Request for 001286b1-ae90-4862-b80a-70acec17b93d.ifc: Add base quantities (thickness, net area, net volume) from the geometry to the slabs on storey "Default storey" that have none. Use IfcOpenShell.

First a look at what the model holds.

```python
import ifcopenshell
import ifcopenshell.util.element
import ifcopenshell.util.unit

model = ifcopenshell.open("001286b1-ae90-4862-b80a-70acec17b93d.ifc")
print(model.schema)
for unit_type in ("LENGTHUNIT", "AREAUNIT", "VOLUMEUNIT"):
    print(unit_type, ifcopenshell.util.unit.calculate_unit_scale(model, unit_type))
storey = next(s for s in model.by_type("IfcBuildingStorey") if s.Name == "Default storey")
slabs = [e for e in ifcopenshell.util.element.get_decomposition(storey) if e.is_a("IfcSlab")]
for e in sorted(slabs, key=lambda e: e.id()):
    print(e.id(), e.is_a(), e.Name, list(ifcopenshell.util.element.get_psets(e, qtos_only=True)), sep=" | ")
```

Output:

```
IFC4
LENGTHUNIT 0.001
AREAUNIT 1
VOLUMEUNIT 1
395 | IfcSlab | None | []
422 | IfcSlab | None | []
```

```python
import ifcopenshell
import ifcopenshell.api.pset
import ifcopenshell.geom
import ifcopenshell.util.element
import ifcopenshell.util.shape
import ifcopenshell.util.unit

model = ifcopenshell.open("001286b1-ae90-4862-b80a-70acec17b93d.ifc")
unit_scale = ifcopenshell.util.unit.calculate_unit_scale(model)
area_scale = ifcopenshell.util.unit.calculate_unit_scale(model, "AREAUNIT")
volume_scale = ifcopenshell.util.unit.calculate_unit_scale(model, "VOLUMEUNIT")
settings = ifcopenshell.geom.settings()

storey = next(s for s in model.by_type("IfcBuildingStorey") if s.Name == "Default storey")
slabs = [e for e in ifcopenshell.util.element.get_decomposition(storey) if e.is_a("IfcSlab")]

for e in sorted(slabs, key=lambda e: e.id()):
    if ifcopenshell.util.element.get_psets(e, qtos_only=True, should_inherit=False):
        continue
    # Geometry comes back in metres, in the element's own axes.
    shape = ifcopenshell.geom.create_shape(settings, e)
    values = {
        "Width": ifcopenshell.util.shape.get_z(shape.geometry) / unit_scale,
        "NetArea": ifcopenshell.util.shape.get_footprint_area(shape.geometry) / area_scale,
        "NetVolume": ifcopenshell.util.shape.get_volume(shape.geometry) / volume_scale,
    }
    qto = ifcopenshell.api.pset.add_qto(model, product=e, name="Qto_SlabBaseQuantities")
    ifcopenshell.api.pset.edit_qto(model, qto=qto, properties=values)
    print(e.id(), {k: round(v, 3) for k, v in values.items()})

model.write("001286b1-ae90-4862-b80a-70acec17b93d_updated.ifc")
```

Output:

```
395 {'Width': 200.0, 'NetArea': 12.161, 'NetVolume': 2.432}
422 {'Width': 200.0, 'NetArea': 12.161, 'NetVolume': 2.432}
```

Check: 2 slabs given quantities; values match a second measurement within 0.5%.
